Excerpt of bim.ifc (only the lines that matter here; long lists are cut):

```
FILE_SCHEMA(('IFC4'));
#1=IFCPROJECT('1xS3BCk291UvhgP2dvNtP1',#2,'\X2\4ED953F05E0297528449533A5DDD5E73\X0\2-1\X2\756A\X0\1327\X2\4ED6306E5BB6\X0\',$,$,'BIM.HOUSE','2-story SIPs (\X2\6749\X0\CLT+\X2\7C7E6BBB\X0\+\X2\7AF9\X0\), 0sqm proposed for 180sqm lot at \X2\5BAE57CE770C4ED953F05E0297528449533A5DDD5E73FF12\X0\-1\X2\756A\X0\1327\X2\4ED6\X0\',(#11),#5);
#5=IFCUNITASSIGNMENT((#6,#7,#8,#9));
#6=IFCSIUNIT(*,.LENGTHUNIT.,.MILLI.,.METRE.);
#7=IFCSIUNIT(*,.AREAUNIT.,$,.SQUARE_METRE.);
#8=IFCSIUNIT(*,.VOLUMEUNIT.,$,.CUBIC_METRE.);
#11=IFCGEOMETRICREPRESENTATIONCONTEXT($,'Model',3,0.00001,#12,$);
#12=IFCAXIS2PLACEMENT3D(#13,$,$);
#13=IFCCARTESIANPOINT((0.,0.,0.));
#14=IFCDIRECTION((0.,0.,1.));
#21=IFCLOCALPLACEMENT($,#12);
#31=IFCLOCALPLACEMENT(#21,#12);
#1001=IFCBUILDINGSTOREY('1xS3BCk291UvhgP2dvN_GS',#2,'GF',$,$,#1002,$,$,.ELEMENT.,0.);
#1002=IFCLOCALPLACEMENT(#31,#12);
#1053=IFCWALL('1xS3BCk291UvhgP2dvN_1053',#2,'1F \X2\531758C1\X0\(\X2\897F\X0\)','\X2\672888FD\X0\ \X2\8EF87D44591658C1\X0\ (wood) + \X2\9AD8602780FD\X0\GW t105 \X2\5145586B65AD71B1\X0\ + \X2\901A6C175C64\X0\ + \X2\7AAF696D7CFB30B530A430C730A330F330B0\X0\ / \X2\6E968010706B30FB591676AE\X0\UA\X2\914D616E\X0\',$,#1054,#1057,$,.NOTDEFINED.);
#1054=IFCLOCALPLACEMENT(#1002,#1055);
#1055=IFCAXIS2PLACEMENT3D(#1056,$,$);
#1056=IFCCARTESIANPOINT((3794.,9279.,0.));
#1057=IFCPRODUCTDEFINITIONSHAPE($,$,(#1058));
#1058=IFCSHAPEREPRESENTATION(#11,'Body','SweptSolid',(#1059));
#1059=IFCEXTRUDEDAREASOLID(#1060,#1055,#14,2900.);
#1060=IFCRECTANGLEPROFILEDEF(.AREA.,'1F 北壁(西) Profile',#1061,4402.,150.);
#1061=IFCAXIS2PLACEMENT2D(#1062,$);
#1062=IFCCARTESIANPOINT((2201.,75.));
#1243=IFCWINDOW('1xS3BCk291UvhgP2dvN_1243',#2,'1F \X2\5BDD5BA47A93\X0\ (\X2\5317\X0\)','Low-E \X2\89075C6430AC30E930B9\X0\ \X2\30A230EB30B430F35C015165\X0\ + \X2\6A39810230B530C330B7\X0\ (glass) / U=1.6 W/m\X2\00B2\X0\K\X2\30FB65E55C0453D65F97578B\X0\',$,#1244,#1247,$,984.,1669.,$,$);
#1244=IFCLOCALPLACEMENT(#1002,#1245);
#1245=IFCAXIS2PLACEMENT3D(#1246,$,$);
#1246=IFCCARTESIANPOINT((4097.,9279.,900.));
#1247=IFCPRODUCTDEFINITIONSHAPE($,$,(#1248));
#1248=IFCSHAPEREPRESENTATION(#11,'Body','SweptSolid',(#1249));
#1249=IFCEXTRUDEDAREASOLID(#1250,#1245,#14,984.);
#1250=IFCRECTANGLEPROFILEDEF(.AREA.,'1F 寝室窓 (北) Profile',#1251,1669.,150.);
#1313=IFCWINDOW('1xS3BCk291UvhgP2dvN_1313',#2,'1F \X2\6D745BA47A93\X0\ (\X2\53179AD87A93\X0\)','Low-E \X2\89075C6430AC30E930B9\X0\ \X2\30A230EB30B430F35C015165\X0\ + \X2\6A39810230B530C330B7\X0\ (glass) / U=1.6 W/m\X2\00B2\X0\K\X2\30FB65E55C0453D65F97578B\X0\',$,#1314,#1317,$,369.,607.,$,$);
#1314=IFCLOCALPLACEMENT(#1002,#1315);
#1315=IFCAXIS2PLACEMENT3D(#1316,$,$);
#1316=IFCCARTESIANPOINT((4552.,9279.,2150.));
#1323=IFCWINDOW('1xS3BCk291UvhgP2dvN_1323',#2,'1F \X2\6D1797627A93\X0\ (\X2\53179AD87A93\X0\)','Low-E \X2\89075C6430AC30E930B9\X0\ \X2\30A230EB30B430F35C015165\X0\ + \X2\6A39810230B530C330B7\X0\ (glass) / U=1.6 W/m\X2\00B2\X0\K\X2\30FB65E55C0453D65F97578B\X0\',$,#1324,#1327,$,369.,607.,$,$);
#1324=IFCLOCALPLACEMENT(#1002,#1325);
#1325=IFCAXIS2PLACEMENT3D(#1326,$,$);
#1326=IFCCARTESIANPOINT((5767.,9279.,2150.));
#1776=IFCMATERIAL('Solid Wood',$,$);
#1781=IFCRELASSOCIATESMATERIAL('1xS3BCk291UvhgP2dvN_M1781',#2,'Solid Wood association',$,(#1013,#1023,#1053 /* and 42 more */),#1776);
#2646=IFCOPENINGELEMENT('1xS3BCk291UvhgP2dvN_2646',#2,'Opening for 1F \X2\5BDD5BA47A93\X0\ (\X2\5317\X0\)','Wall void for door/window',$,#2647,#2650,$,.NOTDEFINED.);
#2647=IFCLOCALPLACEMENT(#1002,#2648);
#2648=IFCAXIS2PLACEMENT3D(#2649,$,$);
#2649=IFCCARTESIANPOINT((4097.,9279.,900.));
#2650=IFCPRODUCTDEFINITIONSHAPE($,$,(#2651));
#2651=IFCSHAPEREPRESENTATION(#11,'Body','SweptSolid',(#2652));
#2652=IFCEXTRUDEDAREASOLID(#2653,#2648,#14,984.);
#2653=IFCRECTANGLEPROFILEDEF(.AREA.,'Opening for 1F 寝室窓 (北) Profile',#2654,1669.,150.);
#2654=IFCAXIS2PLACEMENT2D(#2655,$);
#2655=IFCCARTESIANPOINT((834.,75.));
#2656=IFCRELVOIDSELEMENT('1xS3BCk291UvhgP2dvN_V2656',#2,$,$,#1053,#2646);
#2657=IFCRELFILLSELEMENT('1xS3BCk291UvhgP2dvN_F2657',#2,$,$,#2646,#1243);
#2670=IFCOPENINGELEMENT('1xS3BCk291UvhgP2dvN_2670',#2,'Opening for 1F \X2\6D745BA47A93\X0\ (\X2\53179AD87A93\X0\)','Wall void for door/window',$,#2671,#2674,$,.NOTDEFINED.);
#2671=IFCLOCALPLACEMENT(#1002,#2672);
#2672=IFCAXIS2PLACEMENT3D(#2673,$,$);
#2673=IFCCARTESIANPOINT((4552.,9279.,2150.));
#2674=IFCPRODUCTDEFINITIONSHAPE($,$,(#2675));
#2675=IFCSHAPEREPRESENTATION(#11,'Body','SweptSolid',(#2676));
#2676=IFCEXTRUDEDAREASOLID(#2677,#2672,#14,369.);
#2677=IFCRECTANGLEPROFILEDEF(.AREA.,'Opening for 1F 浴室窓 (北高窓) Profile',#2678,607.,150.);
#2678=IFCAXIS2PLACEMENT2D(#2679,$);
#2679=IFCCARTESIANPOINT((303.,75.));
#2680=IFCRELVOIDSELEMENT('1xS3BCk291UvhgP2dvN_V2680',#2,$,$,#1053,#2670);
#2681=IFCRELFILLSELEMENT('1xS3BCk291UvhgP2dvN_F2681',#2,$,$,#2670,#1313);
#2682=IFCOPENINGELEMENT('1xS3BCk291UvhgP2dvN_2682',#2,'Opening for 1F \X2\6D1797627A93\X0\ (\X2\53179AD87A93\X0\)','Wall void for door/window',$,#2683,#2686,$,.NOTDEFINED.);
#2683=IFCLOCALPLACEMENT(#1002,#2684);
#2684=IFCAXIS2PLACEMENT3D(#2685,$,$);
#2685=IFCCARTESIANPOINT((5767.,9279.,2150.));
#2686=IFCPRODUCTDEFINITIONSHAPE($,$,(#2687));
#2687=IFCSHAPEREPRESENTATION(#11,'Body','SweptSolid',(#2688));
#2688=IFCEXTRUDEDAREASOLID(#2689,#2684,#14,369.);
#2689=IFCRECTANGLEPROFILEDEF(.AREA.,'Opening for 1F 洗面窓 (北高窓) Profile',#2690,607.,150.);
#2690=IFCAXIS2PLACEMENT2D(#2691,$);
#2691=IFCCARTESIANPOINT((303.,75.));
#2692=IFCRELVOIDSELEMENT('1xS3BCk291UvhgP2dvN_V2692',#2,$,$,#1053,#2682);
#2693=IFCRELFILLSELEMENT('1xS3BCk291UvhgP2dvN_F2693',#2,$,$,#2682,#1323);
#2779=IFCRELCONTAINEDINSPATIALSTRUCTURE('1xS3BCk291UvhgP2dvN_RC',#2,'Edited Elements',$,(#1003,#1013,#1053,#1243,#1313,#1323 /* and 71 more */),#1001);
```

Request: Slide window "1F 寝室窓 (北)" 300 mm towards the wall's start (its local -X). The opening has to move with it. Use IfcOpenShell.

```python
import ifcopenshell
import ifcopenshell.api.geometry
import ifcopenshell.util.placement
import ifcopenshell.util.unit

model = ifcopenshell.open("bim.ifc")
unit_scale = ifcopenshell.util.unit.calculate_unit_scale(model)

window = model.by_guid("1xS3BCk291UvhgP2dvN_1243")
opening = window.FillsVoids[0].RelatingOpeningElement
wall = opening.VoidsElements[0].RelatingBuildingElement

wall_matrix = ifcopenshell.util.placement.get_local_placement(wall.ObjectPlacement)
shift = wall_matrix[:3, 0] * -0.3 / unit_scale
before = ifcopenshell.util.placement.get_local_placement(window.ObjectPlacement)[:3, 3].copy()

# The window is not placed relative to its opening, so move both.
for product in (opening, window):
    matrix = ifcopenshell.util.placement.get_local_placement(product.ObjectPlacement)
    matrix[:3, 3] += shift
    ifcopenshell.api.geometry.edit_object_placement(model, product=product, matrix=matrix, is_si=False)

after = ifcopenshell.util.placement.get_local_placement(window.ObjectPlacement)[:3, 3]
print("window moved by", (after - before).round(3) + 0.0)

model.write("bim_updated.ifc")
```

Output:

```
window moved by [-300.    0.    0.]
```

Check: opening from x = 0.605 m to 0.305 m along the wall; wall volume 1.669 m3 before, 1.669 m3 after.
